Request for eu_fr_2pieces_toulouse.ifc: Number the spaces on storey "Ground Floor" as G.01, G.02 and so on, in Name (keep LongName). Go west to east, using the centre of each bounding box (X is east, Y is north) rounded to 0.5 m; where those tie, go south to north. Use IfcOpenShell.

First a look at what the model holds.

```python
import ifcopenshell
import ifcopenshell.util.element
import ifcopenshell.util.placement

model = ifcopenshell.open("eu_fr_2pieces_toulouse.ifc")
print(model.schema)
storey = next(s for s in model.by_type("IfcBuildingStorey") if s.Name == "Ground Floor")
spaces = [e for e in ifcopenshell.util.element.get_decomposition(storey) if e.is_a("IfcSpace")]
for e in sorted(spaces, key=lambda e: e.id()):
    origin = ifcopenshell.util.placement.get_local_placement(e.ObjectPlacement)[:3, 3]
    print(e.id(), e.Name, e.LongName, origin.round(2) + 0.0, sep=" | ")
```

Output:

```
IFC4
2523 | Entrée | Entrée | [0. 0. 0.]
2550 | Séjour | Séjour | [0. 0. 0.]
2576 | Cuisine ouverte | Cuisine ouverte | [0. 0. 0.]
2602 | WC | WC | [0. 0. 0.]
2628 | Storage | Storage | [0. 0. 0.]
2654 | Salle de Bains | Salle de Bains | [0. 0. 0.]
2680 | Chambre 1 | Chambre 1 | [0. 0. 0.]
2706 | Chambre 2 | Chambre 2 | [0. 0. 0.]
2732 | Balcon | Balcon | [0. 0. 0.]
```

```python
import ifcopenshell
import ifcopenshell.geom
import ifcopenshell.util.element
import ifcopenshell.util.shape

model = ifcopenshell.open("eu_fr_2pieces_toulouse.ifc")
settings = ifcopenshell.geom.settings()
settings.set("use-world-coords", True)


def centre(element):
    shape = ifcopenshell.geom.create_shape(settings, element)
    return ifcopenshell.util.shape.get_bbox_centroid(shape.geometry)


storey = next(s for s in model.by_type("IfcBuildingStorey") if s.Name == "Ground Floor")
spaces = [e for e in ifcopenshell.util.element.get_decomposition(storey) if e.is_a("IfcSpace")]

# Insertion points can sit at a corner or the storey origin, so sort by the geometry (in metres).
centres = {e: centre(e) for e in spaces}
spaces.sort(key=lambda e: (round(centres[e][0] / 0.5), centres[e][1]))

for i, e in enumerate(spaces, start=1):
    number = f"G.{i:02d}"
    e.Name = number
    print(e.id(), number)

model.write("eu_fr_2pieces_toulouse_edited.ifc")
```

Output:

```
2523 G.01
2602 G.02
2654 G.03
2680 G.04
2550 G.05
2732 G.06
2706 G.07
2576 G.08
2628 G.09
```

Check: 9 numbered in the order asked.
